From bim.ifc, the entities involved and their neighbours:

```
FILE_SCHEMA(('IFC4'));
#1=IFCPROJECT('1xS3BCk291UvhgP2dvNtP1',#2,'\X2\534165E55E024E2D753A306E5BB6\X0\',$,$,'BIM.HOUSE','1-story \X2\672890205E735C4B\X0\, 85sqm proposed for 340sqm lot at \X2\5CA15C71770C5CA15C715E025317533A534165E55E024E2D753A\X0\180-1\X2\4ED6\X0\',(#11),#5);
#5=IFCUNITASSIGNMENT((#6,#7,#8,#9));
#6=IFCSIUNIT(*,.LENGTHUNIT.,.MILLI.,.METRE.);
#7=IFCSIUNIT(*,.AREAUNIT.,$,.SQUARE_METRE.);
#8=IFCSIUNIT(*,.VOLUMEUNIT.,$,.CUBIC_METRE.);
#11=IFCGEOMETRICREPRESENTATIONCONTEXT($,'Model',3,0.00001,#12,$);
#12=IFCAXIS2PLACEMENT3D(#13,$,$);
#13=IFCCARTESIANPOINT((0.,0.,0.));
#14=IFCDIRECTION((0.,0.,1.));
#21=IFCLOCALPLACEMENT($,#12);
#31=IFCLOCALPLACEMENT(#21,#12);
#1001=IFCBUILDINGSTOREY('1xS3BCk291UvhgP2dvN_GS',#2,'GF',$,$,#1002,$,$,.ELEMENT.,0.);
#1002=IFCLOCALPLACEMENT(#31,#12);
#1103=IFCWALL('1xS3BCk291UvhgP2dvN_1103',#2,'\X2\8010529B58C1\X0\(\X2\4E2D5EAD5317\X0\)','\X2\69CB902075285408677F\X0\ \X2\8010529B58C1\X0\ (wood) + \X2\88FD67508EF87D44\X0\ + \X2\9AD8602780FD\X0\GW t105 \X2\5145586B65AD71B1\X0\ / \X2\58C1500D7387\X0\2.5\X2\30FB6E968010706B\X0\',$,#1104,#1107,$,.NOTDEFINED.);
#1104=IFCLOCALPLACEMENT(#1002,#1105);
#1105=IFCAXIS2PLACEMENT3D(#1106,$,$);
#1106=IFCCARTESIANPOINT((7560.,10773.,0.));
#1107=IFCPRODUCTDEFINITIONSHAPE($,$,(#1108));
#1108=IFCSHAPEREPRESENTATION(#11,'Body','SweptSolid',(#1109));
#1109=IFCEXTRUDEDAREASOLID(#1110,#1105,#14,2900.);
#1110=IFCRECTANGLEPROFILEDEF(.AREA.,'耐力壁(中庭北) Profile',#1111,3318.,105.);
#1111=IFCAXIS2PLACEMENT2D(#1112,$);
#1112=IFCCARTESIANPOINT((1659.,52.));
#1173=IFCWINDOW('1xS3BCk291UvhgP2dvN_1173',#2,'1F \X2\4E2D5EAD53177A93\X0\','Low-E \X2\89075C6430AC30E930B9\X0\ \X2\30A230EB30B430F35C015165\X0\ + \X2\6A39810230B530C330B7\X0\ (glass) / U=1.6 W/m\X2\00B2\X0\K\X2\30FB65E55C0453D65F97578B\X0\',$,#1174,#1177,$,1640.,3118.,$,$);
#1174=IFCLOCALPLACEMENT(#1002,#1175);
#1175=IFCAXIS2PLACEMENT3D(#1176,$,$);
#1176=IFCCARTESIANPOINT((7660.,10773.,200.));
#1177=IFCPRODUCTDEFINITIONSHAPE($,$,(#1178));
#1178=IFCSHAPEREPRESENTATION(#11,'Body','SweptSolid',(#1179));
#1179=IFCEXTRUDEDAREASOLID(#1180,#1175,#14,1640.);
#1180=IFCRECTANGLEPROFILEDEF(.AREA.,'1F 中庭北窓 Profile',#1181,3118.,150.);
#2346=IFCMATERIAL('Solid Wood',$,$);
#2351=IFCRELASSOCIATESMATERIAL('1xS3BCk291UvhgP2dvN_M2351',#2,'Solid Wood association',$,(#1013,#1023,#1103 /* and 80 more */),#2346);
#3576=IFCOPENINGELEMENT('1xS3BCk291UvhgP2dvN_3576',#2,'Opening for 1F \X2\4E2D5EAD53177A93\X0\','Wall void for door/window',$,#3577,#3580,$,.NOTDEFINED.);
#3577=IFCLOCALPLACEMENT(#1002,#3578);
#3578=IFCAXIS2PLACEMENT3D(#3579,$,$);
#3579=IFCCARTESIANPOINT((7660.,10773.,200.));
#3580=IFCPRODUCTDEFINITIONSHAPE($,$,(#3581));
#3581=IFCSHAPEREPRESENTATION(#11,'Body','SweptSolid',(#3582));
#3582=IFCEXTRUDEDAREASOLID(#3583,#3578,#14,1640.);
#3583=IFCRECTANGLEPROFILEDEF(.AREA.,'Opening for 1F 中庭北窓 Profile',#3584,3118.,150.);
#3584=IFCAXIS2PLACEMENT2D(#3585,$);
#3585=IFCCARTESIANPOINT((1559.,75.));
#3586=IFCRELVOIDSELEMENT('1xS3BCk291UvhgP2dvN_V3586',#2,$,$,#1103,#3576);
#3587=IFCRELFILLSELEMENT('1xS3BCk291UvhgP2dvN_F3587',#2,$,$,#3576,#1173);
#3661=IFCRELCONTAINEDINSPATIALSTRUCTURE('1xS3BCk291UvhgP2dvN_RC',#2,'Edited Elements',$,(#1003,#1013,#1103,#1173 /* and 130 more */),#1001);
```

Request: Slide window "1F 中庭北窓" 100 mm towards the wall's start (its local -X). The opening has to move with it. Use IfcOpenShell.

```python
import ifcopenshell
import ifcopenshell.api.geometry
import ifcopenshell.util.placement

model = ifcopenshell.open("bim.ifc")

window = model.by_guid("1xS3BCk291UvhgP2dvN_1173")
opening = window.FillsVoids[0].RelatingOpeningElement
wall = opening.VoidsElements[0].RelatingBuildingElement

wall_matrix = ifcopenshell.util.placement.get_local_placement(wall.ObjectPlacement)
shift = wall_matrix[:3, 0] * -100.0
before = ifcopenshell.util.placement.get_local_placement(window.ObjectPlacement)[:3, 3].copy()

# The window is not placed relative to its opening, so move both.
for product in (opening, window):
    matrix = ifcopenshell.util.placement.get_local_placement(product.ObjectPlacement)
    matrix[:3, 3] += shift
    ifcopenshell.api.geometry.edit_object_placement(model, product=product, matrix=matrix, is_si=False)

after = ifcopenshell.util.placement.get_local_placement(window.ObjectPlacement)[:3, 3]
print("window moved by", (after - before).round(3) + 0.0)

model.write("bim_edited.ifc")
```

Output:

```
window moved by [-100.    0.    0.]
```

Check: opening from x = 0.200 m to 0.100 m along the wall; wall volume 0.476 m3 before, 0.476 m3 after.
